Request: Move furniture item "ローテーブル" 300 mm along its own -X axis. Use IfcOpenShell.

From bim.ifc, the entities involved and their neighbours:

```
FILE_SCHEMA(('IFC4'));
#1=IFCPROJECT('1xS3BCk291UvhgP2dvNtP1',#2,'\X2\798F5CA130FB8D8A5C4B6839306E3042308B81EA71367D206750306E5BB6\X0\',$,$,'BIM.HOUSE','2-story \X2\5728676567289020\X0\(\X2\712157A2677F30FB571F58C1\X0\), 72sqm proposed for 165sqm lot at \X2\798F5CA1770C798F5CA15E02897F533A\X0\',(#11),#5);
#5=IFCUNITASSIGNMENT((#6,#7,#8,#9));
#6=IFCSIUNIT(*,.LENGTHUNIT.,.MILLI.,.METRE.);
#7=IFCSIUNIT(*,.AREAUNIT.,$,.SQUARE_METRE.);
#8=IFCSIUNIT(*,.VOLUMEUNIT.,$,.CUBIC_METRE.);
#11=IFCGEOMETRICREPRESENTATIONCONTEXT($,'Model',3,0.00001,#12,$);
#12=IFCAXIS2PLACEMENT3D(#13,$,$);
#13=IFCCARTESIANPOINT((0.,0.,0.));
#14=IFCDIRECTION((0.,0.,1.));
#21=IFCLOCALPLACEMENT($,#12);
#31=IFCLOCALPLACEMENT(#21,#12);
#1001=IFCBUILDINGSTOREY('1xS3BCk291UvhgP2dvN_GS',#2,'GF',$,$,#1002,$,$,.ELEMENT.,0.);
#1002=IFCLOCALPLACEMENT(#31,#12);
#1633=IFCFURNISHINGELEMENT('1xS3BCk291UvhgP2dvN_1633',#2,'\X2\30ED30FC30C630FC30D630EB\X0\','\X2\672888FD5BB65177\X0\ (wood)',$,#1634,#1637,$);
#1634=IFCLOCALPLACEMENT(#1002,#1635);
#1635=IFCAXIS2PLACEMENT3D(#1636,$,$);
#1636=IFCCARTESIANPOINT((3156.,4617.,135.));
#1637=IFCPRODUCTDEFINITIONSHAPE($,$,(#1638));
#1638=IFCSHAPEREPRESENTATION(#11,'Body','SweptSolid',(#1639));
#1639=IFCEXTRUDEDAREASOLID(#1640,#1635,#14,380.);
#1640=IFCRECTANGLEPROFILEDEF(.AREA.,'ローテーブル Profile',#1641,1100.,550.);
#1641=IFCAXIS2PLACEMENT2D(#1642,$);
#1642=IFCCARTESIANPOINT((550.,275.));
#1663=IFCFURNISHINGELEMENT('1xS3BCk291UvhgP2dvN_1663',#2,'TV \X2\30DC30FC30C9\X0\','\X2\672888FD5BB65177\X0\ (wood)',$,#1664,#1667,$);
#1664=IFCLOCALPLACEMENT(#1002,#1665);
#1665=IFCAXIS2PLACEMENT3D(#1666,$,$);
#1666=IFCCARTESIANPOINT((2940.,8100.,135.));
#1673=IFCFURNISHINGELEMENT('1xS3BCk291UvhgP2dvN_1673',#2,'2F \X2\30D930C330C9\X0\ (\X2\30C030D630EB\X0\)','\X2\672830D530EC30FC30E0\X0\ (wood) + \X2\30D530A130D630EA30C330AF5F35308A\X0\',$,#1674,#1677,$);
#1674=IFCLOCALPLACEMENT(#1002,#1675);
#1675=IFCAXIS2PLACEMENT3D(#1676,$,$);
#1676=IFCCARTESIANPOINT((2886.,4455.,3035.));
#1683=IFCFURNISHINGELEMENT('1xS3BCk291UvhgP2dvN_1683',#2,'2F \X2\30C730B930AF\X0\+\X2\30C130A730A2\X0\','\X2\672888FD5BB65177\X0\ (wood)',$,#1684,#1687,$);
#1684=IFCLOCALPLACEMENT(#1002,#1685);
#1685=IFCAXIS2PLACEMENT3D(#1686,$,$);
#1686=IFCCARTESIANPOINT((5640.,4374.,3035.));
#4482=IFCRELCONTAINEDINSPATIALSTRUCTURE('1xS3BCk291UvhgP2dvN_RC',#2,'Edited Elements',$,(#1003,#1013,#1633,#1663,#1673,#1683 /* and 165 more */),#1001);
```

```python
import ifcopenshell
import ifcopenshell.api.geometry
import ifcopenshell.util.placement
import ifcopenshell.util.unit

model = ifcopenshell.open("bim.ifc")
unit_scale = ifcopenshell.util.unit.calculate_unit_scale(model)

item = model.by_guid("1xS3BCk291UvhgP2dvN_1633")
matrix = ifcopenshell.util.placement.get_local_placement(item.ObjectPlacement)
matrix[:3, 3] -= matrix[:3, 0] * 0.3 / unit_scale
ifcopenshell.api.geometry.edit_object_placement(model, product=item, matrix=matrix, is_si=False)

print(ifcopenshell.util.placement.get_local_placement(item.ObjectPlacement).round(3) + 0.0)

model.write("bim_v2.ifc")
```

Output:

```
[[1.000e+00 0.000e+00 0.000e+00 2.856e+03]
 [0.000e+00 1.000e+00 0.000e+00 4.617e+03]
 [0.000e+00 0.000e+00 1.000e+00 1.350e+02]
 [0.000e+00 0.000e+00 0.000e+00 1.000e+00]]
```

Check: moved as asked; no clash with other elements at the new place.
